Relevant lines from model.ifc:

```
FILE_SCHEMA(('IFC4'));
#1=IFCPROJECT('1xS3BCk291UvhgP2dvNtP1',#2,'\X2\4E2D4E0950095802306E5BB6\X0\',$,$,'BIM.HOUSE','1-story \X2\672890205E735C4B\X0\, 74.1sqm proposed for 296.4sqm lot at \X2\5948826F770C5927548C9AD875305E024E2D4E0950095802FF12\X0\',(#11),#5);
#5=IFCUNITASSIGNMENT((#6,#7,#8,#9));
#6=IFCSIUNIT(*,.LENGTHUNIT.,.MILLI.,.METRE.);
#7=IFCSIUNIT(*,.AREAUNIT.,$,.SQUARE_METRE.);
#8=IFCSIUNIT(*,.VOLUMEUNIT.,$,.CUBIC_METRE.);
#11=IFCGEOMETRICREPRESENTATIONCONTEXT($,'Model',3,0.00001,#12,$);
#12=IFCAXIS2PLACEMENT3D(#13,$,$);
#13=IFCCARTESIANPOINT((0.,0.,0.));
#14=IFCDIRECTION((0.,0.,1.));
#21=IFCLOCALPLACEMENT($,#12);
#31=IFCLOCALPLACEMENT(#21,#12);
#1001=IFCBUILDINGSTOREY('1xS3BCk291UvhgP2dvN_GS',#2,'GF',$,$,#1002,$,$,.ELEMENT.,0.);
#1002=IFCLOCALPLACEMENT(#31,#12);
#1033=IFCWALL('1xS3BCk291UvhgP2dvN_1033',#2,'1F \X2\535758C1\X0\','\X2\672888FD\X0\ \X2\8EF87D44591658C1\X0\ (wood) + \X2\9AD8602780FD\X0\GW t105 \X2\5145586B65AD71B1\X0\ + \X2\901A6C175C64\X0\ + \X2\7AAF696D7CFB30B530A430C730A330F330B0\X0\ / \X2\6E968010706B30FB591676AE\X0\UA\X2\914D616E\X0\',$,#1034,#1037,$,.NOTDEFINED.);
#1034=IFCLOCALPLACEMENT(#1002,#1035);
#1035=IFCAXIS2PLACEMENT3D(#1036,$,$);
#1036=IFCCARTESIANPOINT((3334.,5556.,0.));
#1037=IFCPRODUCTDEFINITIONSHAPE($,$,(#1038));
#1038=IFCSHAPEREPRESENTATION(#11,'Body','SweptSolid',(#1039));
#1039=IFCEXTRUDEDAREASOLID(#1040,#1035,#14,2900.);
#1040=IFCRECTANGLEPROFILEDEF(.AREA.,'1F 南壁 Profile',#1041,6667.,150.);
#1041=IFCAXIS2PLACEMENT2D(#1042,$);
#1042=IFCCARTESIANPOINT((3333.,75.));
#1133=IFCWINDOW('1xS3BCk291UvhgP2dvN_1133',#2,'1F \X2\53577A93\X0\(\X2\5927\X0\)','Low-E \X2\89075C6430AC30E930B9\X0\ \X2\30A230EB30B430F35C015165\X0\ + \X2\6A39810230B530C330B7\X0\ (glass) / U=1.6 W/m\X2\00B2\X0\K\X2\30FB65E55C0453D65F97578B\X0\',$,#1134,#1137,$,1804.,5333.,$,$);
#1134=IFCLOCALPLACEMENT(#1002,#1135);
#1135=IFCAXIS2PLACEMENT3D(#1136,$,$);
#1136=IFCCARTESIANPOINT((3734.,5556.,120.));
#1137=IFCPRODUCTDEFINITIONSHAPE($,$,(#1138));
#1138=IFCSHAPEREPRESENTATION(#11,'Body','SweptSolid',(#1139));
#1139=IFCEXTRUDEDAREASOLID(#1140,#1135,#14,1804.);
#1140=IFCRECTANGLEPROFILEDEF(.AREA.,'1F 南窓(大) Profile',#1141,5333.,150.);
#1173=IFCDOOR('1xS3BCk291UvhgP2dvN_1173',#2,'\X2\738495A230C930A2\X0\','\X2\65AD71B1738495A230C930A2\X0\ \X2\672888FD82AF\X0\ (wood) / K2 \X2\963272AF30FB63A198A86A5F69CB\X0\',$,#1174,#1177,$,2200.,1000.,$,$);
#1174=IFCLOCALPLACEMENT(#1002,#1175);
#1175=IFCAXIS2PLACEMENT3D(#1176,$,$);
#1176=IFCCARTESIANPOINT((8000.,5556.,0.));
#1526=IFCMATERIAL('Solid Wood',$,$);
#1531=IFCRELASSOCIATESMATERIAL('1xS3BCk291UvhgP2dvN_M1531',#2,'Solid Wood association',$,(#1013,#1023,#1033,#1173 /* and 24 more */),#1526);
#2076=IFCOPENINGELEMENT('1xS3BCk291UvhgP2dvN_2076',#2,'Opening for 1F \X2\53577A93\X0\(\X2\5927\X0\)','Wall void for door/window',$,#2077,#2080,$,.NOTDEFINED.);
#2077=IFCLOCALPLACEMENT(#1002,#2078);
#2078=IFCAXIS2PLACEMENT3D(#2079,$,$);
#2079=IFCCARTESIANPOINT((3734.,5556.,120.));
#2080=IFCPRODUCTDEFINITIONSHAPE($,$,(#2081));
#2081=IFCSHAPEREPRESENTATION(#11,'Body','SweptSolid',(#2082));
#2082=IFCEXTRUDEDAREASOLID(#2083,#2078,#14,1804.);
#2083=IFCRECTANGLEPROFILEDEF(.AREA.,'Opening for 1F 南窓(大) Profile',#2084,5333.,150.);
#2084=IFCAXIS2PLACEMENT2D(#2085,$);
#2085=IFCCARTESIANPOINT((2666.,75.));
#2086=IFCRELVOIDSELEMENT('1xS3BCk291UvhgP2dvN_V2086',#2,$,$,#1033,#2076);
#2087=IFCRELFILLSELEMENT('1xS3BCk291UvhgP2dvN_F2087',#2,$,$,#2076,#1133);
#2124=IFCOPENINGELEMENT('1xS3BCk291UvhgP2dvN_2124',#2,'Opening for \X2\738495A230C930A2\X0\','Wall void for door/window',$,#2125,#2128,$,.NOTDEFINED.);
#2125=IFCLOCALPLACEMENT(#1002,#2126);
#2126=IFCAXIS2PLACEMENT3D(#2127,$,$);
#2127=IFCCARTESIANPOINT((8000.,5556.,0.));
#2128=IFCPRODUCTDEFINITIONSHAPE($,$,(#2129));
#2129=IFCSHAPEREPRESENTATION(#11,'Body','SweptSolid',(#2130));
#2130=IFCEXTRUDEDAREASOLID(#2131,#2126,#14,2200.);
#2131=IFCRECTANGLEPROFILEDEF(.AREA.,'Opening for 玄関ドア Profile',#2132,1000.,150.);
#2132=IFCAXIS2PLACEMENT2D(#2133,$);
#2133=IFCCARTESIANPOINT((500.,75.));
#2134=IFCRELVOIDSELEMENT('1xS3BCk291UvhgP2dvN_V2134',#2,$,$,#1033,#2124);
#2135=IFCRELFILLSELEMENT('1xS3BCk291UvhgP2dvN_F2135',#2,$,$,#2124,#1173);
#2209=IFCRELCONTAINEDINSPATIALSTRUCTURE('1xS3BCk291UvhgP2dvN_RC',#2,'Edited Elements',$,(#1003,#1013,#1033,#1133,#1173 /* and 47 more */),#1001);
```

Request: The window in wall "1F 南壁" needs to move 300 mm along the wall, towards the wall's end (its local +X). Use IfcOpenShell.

```python
import ifcopenshell
import ifcopenshell.api.geometry
import ifcopenshell.util.placement
import ifcopenshell.util.unit

model = ifcopenshell.open("model.ifc")
unit_scale = ifcopenshell.util.unit.calculate_unit_scale(model)

window = model.by_guid("1xS3BCk291UvhgP2dvN_1133")
opening = window.FillsVoids[0].RelatingOpeningElement
wall = opening.VoidsElements[0].RelatingBuildingElement

wall_matrix = ifcopenshell.util.placement.get_local_placement(wall.ObjectPlacement)
shift = wall_matrix[:3, 0] * 0.3 / unit_scale
before = ifcopenshell.util.placement.get_local_placement(window.ObjectPlacement)[:3, 3].copy()

# The window is not placed relative to its opening, so move both.
for product in (opening, window):
    matrix = ifcopenshell.util.placement.get_local_placement(product.ObjectPlacement)
    matrix[:3, 3] += shift
    ifcopenshell.api.geometry.edit_object_placement(model, product=product, matrix=matrix, is_si=False)

after = ifcopenshell.util.placement.get_local_placement(window.ObjectPlacement)[:3, 3]
print("window moved by", (after - before).round(3) + 0.0)

model.write("model_rev.ifc")
```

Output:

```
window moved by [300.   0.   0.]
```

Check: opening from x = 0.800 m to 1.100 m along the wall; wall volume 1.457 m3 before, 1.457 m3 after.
